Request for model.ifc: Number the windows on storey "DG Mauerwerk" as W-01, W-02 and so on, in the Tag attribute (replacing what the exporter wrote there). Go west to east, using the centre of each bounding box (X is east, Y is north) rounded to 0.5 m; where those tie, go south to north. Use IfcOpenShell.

First a look at what the model holds.

```python
import ifcopenshell
import ifcopenshell.util.element
import ifcopenshell.util.placement

model = ifcopenshell.open("model.ifc")
print(model.schema)
storey = next(s for s in model.by_type("IfcBuildingStorey") if s.Name == "DG Mauerwerk")
windows = [e for e in ifcopenshell.util.element.get_decomposition(storey) if e.is_a("IfcWindow")]
for e in sorted(windows, key=lambda e: e.id()):
    origin = ifcopenshell.util.placement.get_local_placement(e.ObjectPlacement)[:3, 3]
    print(e.id(), e.Tag, e.Name, origin.round(2) + 0.0, sep=" | ")
```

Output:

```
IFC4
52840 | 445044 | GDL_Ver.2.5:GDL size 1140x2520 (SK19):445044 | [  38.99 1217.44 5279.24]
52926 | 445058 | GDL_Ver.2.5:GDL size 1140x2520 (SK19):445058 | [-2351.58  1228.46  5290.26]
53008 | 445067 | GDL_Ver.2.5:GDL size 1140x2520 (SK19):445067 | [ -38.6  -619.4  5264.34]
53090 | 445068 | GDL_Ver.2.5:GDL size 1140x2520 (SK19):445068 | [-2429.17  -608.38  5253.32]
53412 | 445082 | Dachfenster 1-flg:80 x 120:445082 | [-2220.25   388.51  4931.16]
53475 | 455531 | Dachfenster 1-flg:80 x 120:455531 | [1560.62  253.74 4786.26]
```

```python
import ifcopenshell
import ifcopenshell.geom
import ifcopenshell.util.element
import ifcopenshell.util.shape

model = ifcopenshell.open("model.ifc")
settings = ifcopenshell.geom.settings()
settings.set("use-world-coords", True)


def centre(element):
    shape = ifcopenshell.geom.create_shape(settings, element)
    return ifcopenshell.util.shape.get_bbox_centroid(shape.geometry)


storey = next(s for s in model.by_type("IfcBuildingStorey") if s.Name == "DG Mauerwerk")
windows = [e for e in ifcopenshell.util.element.get_decomposition(storey) if e.is_a("IfcWindow")]

# Insertion points can sit at a corner or the storey origin, so sort by the geometry (in metres).
centres = {e: centre(e) for e in windows}
windows.sort(key=lambda e: (round(centres[e][0] / 0.5), centres[e][1]))

for i, e in enumerate(windows, start=1):
    number = f"W-{i:02d}"
    e.Tag = number
    print(e.id(), number)

model.write("model_edited.ifc")
```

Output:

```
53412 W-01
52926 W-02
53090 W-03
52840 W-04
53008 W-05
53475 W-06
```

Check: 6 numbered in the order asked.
